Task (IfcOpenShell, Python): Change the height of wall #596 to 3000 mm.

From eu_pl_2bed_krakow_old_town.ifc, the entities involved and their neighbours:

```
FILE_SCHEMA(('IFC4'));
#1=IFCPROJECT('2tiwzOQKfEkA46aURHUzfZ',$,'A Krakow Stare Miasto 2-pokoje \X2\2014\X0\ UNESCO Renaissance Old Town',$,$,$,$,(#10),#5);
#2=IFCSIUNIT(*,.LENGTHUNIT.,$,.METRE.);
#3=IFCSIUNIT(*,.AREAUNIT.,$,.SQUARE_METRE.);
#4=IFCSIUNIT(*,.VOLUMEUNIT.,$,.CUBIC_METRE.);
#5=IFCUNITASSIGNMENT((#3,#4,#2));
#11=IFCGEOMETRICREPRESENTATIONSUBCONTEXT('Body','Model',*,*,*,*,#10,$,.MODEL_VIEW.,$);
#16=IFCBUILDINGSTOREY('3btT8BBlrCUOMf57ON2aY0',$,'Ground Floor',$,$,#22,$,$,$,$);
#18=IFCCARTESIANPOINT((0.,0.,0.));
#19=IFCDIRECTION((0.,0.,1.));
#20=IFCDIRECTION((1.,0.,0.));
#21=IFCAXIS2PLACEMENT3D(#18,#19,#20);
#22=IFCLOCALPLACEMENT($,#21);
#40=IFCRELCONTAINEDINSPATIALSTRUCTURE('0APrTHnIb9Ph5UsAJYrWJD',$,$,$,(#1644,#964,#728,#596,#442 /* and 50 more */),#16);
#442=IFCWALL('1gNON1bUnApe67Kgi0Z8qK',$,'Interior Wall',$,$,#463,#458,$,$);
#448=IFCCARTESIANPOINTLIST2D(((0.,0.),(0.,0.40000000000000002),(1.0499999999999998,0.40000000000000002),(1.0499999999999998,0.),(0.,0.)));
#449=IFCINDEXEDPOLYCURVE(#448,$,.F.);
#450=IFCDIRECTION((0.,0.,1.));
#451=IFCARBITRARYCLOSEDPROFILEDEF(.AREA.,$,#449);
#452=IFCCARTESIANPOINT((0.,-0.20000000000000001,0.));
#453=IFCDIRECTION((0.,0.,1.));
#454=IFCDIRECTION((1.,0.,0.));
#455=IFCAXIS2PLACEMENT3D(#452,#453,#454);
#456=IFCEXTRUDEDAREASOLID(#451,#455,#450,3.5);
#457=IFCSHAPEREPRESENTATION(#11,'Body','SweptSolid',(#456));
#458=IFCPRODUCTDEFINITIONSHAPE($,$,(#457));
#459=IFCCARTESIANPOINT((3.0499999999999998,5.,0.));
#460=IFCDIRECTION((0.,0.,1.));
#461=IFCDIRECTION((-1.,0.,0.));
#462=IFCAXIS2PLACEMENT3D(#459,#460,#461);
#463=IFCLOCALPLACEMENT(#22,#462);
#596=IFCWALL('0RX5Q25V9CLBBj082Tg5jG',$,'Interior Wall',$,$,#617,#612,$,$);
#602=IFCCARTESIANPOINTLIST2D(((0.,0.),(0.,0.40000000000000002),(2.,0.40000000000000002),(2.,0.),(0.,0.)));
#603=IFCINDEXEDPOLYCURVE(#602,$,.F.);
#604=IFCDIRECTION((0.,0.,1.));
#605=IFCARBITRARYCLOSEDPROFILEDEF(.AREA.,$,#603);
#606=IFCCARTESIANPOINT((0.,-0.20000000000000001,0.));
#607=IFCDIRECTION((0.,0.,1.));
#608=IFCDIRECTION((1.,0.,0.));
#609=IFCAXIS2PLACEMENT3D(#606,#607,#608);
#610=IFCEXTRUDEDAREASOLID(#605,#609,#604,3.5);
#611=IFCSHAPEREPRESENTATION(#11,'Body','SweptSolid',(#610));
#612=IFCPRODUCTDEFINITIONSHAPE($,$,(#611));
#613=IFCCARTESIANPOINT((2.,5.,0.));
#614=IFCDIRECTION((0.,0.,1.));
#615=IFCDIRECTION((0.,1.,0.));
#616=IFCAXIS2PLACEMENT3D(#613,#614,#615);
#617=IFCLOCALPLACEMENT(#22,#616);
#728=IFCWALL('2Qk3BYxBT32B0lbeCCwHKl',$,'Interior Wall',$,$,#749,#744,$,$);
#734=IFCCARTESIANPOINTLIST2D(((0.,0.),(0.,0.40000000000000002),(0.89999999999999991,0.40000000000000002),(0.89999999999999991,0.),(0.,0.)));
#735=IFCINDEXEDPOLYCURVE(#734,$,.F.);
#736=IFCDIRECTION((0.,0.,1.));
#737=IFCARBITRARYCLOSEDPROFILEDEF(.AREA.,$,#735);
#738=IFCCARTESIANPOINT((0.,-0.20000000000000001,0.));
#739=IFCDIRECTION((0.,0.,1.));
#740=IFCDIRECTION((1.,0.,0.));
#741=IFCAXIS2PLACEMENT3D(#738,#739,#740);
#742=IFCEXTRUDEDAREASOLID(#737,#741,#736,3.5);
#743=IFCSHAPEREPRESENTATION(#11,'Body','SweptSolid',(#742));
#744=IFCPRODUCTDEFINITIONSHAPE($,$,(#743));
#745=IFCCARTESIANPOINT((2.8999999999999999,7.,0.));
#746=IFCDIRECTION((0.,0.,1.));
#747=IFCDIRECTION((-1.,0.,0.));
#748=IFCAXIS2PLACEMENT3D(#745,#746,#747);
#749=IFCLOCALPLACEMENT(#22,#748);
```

```python
import ifcopenshell
import ifcopenshell.geom
import ifcopenshell.util.representation
import ifcopenshell.util.shape

model = ifcopenshell.open("eu_pl_2bed_krakow_old_town.ifc")
settings = ifcopenshell.geom.settings()


def volume(element):
    """Net volume in cubic metres, openings subtracted."""
    shape = ifcopenshell.geom.create_shape(settings, element)
    return ifcopenshell.util.shape.get_volume(shape.geometry)


wall = model.by_guid("0RX5Q25V9CLBBj082Tg5jG")
before = volume(wall)

body = ifcopenshell.util.representation.get_representation(wall, "Model", "Body")
solid = body.Items[0]
old_height = solid.Depth
solid.Depth = 3.0
after = volume(wall)

print(f"height {old_height:g} -> {solid.Depth:g}, volume {before:.3f} -> {after:.3f} m3")

model.write("eu_pl_2bed_krakow_old_town-out.ifc")
```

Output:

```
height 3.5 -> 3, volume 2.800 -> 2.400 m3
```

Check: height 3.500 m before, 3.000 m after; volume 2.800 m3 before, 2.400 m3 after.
